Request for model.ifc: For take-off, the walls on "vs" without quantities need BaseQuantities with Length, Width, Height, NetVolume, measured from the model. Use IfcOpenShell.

First a look at what the model holds.

```python
import ifcopenshell
import ifcopenshell.util.element
import ifcopenshell.util.unit

model = ifcopenshell.open("model.ifc")
print(model.schema)
for unit_type in ("LENGTHUNIT", "AREAUNIT", "VOLUMEUNIT"):
    print(unit_type, ifcopenshell.util.unit.calculate_unit_scale(model, unit_type))
storey = next(s for s in model.by_type("IfcBuildingStorey") if s.Name == "vs")
walls = [e for e in ifcopenshell.util.element.get_decomposition(storey) if e.is_a("IfcWall")]
for e in sorted(walls, key=lambda e: e.id()):
    print(e.id(), e.is_a(), e.Name, list(ifcopenshell.util.element.get_psets(e, qtos_only=True)), sep=" | ")
```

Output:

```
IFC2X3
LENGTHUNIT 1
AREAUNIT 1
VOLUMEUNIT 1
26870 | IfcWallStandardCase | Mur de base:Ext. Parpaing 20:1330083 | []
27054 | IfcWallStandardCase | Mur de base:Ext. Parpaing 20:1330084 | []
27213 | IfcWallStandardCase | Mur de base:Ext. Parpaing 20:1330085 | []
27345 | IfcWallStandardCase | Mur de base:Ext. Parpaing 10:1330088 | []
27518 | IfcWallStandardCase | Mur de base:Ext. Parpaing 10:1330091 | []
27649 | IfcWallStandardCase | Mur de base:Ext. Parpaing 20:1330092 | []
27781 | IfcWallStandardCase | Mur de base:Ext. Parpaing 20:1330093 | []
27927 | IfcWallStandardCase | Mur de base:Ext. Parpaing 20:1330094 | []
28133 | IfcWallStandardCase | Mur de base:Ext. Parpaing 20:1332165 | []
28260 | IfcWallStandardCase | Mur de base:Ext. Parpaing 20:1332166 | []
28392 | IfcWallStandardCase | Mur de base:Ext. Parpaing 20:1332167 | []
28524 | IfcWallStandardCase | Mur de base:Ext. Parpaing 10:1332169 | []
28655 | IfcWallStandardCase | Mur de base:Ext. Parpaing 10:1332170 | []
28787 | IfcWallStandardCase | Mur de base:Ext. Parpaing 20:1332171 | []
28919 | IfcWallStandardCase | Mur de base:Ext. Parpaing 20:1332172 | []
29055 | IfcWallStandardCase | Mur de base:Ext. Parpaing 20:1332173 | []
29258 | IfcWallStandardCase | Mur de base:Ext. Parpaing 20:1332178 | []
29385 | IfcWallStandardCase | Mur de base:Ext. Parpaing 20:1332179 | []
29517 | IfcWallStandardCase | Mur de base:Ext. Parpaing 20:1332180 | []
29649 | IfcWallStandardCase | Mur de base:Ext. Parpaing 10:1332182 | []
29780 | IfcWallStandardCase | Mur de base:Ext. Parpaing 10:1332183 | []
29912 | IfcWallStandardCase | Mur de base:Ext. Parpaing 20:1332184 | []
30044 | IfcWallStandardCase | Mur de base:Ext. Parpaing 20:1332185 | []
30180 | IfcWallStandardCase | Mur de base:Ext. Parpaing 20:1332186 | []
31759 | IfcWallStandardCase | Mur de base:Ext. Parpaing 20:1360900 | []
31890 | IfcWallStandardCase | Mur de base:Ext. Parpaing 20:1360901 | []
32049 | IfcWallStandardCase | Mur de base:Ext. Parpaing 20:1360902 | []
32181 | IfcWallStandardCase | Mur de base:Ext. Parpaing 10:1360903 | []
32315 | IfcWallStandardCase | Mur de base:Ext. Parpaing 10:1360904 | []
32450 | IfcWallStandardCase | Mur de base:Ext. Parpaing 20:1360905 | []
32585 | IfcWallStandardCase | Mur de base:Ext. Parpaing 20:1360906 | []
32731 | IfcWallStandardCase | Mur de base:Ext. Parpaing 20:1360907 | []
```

```python
import ifcopenshell
import ifcopenshell.api.pset
import ifcopenshell.geom
import ifcopenshell.util.element
import ifcopenshell.util.shape
import ifcopenshell.util.unit

model = ifcopenshell.open("model.ifc")
unit_scale = ifcopenshell.util.unit.calculate_unit_scale(model)
volume_scale = ifcopenshell.util.unit.calculate_unit_scale(model, "VOLUMEUNIT")
settings = ifcopenshell.geom.settings()

storey = next(s for s in model.by_type("IfcBuildingStorey") if s.Name == "vs")
walls = [e for e in ifcopenshell.util.element.get_decomposition(storey) if e.is_a("IfcWall")]

for e in sorted(walls, key=lambda e: e.id()):
    if ifcopenshell.util.element.get_psets(e, qtos_only=True, should_inherit=False):
        continue
    # Geometry comes back in metres, in the element's own axes.
    shape = ifcopenshell.geom.create_shape(settings, e)
    values = {
        "Length": ifcopenshell.util.shape.get_x(shape.geometry) / unit_scale,
        "Width": ifcopenshell.util.shape.get_y(shape.geometry) / unit_scale,
        "Height": ifcopenshell.util.shape.get_z(shape.geometry) / unit_scale,
        "NetVolume": ifcopenshell.util.shape.get_volume(shape.geometry) / volume_scale,
    }
    qto = ifcopenshell.api.pset.add_qto(model, product=e, name="BaseQuantities")
    ifcopenshell.api.pset.edit_qto(model, qto=qto, properties=values)
    print(e.id(), {k: round(v, 3) for k, v in values.items()})

model.write("model_v2.ifc")
```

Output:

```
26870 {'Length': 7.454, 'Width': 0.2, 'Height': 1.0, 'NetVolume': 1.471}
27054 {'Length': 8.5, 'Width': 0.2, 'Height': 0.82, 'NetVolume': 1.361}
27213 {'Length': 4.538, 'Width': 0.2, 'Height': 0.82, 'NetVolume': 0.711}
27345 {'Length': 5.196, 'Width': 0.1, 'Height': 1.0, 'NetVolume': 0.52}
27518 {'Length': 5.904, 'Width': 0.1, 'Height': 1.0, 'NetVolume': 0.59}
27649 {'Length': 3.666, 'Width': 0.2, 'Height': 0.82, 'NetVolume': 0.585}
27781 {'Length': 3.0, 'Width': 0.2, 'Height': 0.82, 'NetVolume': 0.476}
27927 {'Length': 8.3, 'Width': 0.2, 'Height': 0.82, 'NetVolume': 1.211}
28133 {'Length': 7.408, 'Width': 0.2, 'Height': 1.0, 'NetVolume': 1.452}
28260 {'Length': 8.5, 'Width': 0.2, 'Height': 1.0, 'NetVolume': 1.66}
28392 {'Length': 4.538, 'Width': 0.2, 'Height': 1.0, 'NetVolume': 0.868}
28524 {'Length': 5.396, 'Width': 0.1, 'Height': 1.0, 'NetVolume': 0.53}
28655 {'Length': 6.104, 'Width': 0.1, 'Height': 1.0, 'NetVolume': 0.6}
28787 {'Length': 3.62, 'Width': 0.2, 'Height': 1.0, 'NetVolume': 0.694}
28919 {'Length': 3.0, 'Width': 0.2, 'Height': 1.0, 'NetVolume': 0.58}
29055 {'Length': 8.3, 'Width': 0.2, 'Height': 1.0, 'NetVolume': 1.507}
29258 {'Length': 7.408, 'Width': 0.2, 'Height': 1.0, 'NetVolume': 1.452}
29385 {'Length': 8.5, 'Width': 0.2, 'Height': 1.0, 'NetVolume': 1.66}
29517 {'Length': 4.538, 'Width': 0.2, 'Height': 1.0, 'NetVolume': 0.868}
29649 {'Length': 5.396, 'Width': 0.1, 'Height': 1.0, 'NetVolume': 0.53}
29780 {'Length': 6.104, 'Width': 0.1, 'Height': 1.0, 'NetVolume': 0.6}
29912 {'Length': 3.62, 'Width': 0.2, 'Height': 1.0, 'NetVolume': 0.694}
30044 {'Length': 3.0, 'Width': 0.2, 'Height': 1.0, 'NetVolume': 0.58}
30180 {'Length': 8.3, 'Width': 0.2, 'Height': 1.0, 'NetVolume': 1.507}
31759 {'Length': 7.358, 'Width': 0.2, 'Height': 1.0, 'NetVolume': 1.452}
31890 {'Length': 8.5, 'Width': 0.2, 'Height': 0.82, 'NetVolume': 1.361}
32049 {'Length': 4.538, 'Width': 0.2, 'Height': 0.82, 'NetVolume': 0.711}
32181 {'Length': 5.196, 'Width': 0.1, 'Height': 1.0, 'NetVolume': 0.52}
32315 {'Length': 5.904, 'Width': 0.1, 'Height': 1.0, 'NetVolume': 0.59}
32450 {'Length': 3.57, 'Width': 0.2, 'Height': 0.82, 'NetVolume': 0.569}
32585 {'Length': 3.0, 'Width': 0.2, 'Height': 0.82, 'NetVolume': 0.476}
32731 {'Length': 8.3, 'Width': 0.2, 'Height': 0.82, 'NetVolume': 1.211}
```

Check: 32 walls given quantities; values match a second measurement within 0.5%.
